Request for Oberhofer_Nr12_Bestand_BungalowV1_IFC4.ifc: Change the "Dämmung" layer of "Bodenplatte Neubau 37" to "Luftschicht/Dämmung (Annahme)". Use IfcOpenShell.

First a look at what the model holds.

```python
import ifcopenshell
import ifcopenshell.util.element

model = ifcopenshell.open("Oberhofer_Nr12_Bestand_BungalowV1_IFC4.ifc")
print(model.schema)
for layer_set in model.by_type("IfcMaterialLayerSet"):
    if layer_set.LayerSetName == "Bodenplatte Neubau 37":
        for layer in layer_set.MaterialLayers:
            print(layer.id(), layer.Material and layer.Material.Name, layer.LayerThickness, sep=" | ")
        print(len(ifcopenshell.util.element.get_elements_by_material(model, layer_set)), "elements and types use it")
print(sorted(m.Name for m in model.by_type("IfcMaterial") if m.Name)[:60])
```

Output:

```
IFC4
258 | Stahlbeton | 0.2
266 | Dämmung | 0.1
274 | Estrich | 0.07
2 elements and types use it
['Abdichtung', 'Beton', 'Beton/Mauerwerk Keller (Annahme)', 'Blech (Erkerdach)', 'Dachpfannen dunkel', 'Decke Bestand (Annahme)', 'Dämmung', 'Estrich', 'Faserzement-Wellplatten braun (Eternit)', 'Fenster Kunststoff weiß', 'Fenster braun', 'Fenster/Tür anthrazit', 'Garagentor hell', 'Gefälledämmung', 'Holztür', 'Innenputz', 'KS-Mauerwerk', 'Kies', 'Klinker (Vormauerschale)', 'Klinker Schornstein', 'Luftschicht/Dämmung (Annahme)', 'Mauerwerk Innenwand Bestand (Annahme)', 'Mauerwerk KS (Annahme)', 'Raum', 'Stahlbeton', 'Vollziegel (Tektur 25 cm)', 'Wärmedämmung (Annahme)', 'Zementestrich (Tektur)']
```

```python
import ifcopenshell
import ifcopenshell.api.material

model = ifcopenshell.open("Oberhofer_Nr12_Bestand_BungalowV1_IFC4.ifc")

layer_set = next(s for s in model.by_type("IfcMaterialLayerSet") if s.LayerSetName == "Bodenplatte Neubau 37")
layer = next(l for l in layer_set.MaterialLayers if l.Material and l.Material.Name == "Dämmung")
material = next(m for m in model.by_type("IfcMaterial") if m.Name == "Luftschicht/Dämmung (Annahme)")

# Point this one layer at the other material; renaming the old one would change it everywhere.
ifcopenshell.api.material.edit_layer(model, layer=layer, attributes={}, material=material)

print([l.Material.Name if l.Material else None for l in layer_set.MaterialLayers])

model.write("Oberhofer_Nr12_Bestand_BungalowV1_IFC4-out.ifc")
```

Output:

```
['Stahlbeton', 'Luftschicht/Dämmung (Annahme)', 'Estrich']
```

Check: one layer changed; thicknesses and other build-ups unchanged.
